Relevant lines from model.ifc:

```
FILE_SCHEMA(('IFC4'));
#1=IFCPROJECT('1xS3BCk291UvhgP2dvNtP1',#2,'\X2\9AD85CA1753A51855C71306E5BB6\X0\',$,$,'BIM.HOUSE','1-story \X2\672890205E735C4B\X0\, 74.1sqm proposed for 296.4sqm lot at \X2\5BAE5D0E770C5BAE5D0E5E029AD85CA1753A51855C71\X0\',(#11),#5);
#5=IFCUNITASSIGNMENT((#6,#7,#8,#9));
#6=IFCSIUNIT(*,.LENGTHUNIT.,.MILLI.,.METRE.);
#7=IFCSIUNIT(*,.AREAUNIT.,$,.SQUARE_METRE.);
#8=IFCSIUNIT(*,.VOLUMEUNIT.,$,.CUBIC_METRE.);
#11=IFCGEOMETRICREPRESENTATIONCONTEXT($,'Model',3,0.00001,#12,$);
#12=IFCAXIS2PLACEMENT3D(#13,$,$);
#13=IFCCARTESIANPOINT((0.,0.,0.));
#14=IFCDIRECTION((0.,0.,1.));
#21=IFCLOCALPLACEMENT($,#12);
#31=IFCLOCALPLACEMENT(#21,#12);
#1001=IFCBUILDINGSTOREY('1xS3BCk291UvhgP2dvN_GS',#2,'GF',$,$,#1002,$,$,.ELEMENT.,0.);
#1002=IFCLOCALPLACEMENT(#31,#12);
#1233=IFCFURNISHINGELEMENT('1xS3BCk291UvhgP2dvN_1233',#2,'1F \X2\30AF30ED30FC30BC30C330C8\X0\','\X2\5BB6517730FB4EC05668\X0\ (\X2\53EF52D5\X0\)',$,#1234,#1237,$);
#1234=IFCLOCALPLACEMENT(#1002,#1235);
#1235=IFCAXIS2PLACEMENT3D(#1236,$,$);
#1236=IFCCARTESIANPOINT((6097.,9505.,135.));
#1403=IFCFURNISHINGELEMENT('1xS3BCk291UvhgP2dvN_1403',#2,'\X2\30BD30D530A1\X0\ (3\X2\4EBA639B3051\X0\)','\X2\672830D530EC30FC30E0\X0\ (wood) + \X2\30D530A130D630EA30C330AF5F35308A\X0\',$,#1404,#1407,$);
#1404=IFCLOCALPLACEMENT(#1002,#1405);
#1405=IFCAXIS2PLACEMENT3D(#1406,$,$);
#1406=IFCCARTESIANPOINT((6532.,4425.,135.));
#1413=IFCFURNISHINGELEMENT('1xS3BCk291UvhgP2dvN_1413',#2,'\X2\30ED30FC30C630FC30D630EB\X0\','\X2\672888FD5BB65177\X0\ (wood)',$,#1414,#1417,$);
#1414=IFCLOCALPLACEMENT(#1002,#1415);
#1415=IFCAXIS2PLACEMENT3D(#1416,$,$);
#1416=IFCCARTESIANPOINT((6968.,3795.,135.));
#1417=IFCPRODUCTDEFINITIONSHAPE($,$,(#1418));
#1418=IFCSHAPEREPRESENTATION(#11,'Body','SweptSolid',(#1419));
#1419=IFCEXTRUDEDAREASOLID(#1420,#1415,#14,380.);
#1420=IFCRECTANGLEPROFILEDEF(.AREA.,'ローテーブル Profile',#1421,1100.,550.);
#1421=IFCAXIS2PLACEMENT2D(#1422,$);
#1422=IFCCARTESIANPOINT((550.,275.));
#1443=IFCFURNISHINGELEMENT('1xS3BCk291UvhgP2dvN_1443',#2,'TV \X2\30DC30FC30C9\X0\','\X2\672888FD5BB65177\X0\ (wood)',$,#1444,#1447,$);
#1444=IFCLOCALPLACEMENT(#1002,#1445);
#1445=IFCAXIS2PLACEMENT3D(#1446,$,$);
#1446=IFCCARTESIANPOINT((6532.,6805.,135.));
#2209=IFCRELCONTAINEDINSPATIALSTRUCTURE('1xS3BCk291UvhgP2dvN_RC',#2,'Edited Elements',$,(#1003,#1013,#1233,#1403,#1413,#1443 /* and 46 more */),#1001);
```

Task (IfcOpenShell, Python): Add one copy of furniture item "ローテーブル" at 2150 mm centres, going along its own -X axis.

```python
import ifcopenshell
import ifcopenshell.api.geometry
import ifcopenshell.api.root
import ifcopenshell.util.element
import ifcopenshell.util.placement
import ifcopenshell.util.unit

model = ifcopenshell.open("model.ifc")
unit_scale = ifcopenshell.util.unit.calculate_unit_scale(model)


def reuse_history(source, copy):
    """copy_class also copies each property set's owner history, people and application; keep the originals."""
    for rel in copy.IsDefinedBy:
        if rel.is_a("IfcRelDefinesByProperties") and (history := rel.RelatingPropertyDefinition.OwnerHistory):
            rel.RelatingPropertyDefinition.OwnerHistory = source.OwnerHistory
            ifcopenshell.util.element.remove_deep2(model, history)


source = model.by_guid("1xS3BCk291UvhgP2dvN_1413")
base = ifcopenshell.util.placement.get_local_placement(source.ObjectPlacement)
step = -base[:3, 0] * 2.15 / unit_scale

for i in range(1, 2):
    copy = ifcopenshell.api.root.copy_class(model, product=source)
    copy.Representation = ifcopenshell.util.element.copy_deep(
        model, source.Representation, exclude=["IfcGeometricRepresentationContext", "IfcRepresentationMap"]
    )
    reuse_history(source, copy)
    matrix = base.copy()
    matrix[:3, 3] += i * step
    print("added at", matrix[:3, 3].round(3) + 0.0)
    ifcopenshell.api.geometry.edit_object_placement(model, product=copy, matrix=matrix, is_si=False)

model.write("model_edited.ifc")
```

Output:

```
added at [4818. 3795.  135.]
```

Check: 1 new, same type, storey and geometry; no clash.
